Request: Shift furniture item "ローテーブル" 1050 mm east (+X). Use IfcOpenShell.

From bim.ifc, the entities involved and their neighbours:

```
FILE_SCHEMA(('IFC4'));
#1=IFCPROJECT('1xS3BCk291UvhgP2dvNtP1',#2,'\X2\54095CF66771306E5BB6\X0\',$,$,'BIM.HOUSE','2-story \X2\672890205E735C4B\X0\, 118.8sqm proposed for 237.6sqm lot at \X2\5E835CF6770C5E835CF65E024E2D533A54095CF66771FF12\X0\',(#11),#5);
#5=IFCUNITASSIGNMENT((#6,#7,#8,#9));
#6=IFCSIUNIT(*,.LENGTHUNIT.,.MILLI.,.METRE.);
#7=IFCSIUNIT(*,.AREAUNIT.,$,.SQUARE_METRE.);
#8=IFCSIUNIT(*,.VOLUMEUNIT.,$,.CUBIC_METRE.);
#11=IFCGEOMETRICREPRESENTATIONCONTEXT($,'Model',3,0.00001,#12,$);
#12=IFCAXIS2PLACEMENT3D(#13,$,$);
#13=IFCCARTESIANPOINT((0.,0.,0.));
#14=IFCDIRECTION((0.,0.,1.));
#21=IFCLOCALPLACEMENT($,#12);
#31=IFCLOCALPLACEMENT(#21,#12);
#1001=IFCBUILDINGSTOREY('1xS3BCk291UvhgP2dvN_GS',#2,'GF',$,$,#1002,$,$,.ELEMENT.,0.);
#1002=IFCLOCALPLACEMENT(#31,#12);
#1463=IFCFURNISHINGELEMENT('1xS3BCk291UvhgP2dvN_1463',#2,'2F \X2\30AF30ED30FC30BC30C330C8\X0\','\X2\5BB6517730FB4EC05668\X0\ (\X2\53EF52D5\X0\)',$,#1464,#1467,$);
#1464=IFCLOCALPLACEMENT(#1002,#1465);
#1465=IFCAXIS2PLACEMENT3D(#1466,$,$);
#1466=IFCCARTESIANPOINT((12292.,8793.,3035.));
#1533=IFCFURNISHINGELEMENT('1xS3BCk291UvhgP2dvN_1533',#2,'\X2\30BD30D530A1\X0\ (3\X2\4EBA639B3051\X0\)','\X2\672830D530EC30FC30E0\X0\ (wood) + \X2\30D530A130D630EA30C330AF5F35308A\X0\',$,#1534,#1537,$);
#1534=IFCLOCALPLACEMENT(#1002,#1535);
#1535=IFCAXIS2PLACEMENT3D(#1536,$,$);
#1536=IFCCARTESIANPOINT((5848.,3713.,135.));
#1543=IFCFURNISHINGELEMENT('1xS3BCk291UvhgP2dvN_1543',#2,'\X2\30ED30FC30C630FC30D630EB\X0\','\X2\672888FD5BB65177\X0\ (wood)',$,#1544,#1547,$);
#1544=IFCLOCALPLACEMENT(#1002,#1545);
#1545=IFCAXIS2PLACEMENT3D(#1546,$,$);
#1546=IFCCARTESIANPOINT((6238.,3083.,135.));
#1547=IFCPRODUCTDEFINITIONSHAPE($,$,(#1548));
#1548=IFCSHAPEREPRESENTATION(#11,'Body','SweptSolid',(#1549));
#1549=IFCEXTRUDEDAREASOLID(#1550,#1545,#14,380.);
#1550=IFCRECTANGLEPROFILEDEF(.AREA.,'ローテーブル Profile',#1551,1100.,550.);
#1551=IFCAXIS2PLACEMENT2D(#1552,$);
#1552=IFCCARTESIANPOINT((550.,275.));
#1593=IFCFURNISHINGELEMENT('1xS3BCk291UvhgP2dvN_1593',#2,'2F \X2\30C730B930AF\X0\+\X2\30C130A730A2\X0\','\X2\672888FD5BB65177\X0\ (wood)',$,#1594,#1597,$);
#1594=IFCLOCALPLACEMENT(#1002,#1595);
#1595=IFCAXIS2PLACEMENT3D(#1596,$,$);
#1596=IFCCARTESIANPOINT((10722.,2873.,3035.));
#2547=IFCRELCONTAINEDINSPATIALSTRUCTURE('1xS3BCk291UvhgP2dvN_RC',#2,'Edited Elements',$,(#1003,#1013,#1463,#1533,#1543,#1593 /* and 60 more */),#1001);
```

```python
import ifcopenshell
import ifcopenshell.api.geometry
import ifcopenshell.util.placement
import ifcopenshell.util.unit

model = ifcopenshell.open("bim.ifc")
unit_scale = ifcopenshell.util.unit.calculate_unit_scale(model)

item = model.by_guid("1xS3BCk291UvhgP2dvN_1543")
matrix = ifcopenshell.util.placement.get_local_placement(item.ObjectPlacement)
matrix[0, 3] += 1.05 / unit_scale
ifcopenshell.api.geometry.edit_object_placement(model, product=item, matrix=matrix, is_si=False)

print(ifcopenshell.util.placement.get_local_placement(item.ObjectPlacement).round(3) + 0.0)

model.write("bim-out.ifc")
```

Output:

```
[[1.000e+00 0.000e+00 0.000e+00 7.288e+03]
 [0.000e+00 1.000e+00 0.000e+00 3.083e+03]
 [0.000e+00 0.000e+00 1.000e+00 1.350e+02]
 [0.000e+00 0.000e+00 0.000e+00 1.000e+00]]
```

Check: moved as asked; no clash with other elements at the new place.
